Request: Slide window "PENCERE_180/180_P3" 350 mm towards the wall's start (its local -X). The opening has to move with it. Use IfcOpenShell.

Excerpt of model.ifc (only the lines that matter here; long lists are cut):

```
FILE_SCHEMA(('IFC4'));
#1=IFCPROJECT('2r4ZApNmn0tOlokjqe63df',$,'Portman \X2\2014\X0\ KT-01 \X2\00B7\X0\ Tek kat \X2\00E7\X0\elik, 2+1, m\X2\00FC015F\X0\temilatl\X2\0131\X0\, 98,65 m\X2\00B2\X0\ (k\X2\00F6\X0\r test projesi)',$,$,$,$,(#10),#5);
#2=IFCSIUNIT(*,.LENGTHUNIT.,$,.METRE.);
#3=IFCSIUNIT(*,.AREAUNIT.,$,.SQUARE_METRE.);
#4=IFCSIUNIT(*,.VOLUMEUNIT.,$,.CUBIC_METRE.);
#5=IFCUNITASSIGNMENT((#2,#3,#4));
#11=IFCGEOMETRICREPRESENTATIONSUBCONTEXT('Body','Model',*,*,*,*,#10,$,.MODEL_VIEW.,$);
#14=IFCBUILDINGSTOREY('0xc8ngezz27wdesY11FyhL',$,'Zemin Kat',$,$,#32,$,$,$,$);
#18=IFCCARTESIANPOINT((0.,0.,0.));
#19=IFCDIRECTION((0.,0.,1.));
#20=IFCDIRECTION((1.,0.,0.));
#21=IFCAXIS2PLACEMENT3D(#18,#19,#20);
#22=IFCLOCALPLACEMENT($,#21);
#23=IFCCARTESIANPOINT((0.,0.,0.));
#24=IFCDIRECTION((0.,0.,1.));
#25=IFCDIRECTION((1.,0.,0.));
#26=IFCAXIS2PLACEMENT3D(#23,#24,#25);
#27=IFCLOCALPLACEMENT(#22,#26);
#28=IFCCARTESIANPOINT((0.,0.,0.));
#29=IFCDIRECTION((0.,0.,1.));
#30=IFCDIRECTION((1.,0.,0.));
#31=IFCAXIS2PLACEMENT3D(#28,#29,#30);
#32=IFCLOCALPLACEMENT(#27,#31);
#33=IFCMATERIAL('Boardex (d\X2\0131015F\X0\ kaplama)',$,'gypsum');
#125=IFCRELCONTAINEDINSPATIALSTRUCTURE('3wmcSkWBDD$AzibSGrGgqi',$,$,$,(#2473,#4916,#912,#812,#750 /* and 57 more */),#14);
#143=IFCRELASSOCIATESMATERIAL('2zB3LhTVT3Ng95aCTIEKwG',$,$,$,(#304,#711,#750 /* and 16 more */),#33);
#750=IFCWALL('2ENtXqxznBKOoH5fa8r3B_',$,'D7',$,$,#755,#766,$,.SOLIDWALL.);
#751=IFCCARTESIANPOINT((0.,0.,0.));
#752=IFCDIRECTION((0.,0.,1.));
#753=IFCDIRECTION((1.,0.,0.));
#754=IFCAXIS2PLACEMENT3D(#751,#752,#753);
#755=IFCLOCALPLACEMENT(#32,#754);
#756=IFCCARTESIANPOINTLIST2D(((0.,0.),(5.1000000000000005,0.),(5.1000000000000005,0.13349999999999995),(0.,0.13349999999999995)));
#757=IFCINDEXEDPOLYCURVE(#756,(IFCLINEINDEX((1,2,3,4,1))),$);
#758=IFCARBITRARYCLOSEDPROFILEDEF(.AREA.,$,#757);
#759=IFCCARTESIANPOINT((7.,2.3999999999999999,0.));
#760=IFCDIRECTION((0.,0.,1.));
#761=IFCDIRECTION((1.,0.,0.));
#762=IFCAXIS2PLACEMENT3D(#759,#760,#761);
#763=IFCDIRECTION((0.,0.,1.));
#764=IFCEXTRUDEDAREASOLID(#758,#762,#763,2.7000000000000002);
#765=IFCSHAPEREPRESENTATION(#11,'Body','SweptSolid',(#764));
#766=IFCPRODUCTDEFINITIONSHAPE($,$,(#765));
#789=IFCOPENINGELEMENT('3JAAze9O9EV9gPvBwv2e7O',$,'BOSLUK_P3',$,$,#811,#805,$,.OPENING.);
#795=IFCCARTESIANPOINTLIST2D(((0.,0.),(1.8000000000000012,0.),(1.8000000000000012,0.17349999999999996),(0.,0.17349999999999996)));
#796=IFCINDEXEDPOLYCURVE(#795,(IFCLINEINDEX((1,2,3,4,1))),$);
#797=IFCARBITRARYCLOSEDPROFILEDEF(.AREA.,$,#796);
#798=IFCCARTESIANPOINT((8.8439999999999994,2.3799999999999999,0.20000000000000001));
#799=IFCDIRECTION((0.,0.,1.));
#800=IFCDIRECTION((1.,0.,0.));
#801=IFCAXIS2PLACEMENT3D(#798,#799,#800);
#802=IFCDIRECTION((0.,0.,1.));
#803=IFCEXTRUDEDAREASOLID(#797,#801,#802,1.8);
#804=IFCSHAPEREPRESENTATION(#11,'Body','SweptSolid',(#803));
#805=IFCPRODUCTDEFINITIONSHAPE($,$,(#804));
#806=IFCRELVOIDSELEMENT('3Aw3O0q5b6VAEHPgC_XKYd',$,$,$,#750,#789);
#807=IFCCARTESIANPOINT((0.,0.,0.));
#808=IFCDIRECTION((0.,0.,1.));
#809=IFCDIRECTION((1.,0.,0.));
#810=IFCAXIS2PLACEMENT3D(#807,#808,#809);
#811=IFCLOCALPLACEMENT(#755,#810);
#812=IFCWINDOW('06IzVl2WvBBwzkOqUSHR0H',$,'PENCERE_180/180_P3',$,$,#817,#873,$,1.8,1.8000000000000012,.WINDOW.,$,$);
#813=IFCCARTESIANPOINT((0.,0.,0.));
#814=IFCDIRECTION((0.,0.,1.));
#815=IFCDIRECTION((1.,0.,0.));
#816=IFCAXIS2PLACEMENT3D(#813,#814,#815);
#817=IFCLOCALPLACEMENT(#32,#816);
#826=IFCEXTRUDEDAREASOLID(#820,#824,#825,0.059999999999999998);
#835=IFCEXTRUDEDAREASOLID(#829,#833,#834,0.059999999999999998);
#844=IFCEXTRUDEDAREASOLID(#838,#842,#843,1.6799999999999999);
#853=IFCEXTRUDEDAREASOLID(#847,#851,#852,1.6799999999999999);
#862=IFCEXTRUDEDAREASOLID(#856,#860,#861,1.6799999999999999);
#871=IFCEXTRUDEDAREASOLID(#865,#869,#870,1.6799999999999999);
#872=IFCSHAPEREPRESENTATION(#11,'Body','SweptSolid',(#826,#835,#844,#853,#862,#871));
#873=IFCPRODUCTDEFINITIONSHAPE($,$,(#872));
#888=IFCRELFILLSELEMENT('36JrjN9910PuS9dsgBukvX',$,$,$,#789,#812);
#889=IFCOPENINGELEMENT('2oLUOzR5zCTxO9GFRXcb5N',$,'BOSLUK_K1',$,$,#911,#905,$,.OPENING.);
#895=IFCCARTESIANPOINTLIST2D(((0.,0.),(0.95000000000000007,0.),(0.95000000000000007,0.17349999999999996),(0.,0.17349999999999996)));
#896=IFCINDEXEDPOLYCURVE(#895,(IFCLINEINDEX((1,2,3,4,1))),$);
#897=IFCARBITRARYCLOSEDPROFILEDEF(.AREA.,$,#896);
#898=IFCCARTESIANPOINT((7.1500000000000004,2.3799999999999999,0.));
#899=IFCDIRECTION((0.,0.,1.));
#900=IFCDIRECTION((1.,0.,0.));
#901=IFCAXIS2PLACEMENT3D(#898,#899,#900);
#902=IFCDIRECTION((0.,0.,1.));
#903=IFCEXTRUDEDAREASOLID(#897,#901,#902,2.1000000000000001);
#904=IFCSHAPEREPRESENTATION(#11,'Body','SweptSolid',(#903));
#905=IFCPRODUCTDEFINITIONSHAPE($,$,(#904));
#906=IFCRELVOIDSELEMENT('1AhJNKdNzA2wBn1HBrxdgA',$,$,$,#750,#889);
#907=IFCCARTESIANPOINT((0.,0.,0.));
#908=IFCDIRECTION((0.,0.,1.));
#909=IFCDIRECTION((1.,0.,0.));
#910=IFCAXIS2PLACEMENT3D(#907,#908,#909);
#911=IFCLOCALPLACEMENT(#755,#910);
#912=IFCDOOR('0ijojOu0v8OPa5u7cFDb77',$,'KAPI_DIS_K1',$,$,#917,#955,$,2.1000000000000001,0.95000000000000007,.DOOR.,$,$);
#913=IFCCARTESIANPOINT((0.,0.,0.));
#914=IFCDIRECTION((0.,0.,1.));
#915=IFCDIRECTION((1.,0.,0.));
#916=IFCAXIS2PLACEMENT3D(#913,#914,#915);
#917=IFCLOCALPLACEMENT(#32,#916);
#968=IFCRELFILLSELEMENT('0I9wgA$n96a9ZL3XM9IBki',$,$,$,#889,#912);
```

```python
import ifcopenshell
import ifcopenshell.api.geometry
import ifcopenshell.util.placement
import ifcopenshell.util.unit

model = ifcopenshell.open("model.ifc")
unit_scale = ifcopenshell.util.unit.calculate_unit_scale(model)

window = model.by_id(812)
opening = window.FillsVoids[0].RelatingOpeningElement
wall = opening.VoidsElements[0].RelatingBuildingElement

wall_matrix = ifcopenshell.util.placement.get_local_placement(wall.ObjectPlacement)
shift = wall_matrix[:3, 0] * -0.35 / unit_scale
before = ifcopenshell.util.placement.get_local_placement(window.ObjectPlacement)[:3, 3].copy()

# The window is not placed relative to its opening, so move both.
for product in (opening, window):
    matrix = ifcopenshell.util.placement.get_local_placement(product.ObjectPlacement)
    matrix[:3, 3] += shift
    ifcopenshell.api.geometry.edit_object_placement(model, product=product, matrix=matrix, is_si=False)

after = ifcopenshell.util.placement.get_local_placement(window.ObjectPlacement)[:3, 3]
print("window moved by", (after - before).round(3) + 0.0)

model.write("model_edited.ifc")
```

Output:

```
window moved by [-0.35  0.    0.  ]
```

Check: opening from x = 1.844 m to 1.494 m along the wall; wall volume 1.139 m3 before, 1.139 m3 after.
